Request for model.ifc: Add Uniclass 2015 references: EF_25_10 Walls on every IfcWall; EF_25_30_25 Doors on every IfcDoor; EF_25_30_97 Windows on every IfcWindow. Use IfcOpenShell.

First a look at what the model holds.

```python
import ifcopenshell

model = ifcopenshell.open("model.ifc")
print(model.schema)
print("classifications:", [c.Name for c in model.by_type("IfcClassification")])
for ifc_class in ("IfcDoor", "IfcRoof", "IfcStair", "IfcWall", "IfcWindow"):
    print(ifc_class, len(model.by_type(ifc_class)))
```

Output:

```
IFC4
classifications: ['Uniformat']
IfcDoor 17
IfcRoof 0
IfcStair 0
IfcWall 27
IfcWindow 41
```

```python
import ifcopenshell
import ifcopenshell.api.classification

model = ifcopenshell.open("model.ifc")

system = ifcopenshell.api.classification.add_classification(model, classification="Uniclass 2015")

codes = {
    "IfcWall": ("EF_25_10", "Walls"),
    "IfcDoor": ("EF_25_30_25", "Doors"),
    "IfcWindow": ("EF_25_30_97", "Windows"),
}
for ifc_class, (code, name) in codes.items():
    products = model.by_type(ifc_class)
    ifcopenshell.api.classification.add_reference(
        model, products=products, classification=system, identification=code, name=name
    )
    print(code, len(products))

model.write("model_updated.ifc")
```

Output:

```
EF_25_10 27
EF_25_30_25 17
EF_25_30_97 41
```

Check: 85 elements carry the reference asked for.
